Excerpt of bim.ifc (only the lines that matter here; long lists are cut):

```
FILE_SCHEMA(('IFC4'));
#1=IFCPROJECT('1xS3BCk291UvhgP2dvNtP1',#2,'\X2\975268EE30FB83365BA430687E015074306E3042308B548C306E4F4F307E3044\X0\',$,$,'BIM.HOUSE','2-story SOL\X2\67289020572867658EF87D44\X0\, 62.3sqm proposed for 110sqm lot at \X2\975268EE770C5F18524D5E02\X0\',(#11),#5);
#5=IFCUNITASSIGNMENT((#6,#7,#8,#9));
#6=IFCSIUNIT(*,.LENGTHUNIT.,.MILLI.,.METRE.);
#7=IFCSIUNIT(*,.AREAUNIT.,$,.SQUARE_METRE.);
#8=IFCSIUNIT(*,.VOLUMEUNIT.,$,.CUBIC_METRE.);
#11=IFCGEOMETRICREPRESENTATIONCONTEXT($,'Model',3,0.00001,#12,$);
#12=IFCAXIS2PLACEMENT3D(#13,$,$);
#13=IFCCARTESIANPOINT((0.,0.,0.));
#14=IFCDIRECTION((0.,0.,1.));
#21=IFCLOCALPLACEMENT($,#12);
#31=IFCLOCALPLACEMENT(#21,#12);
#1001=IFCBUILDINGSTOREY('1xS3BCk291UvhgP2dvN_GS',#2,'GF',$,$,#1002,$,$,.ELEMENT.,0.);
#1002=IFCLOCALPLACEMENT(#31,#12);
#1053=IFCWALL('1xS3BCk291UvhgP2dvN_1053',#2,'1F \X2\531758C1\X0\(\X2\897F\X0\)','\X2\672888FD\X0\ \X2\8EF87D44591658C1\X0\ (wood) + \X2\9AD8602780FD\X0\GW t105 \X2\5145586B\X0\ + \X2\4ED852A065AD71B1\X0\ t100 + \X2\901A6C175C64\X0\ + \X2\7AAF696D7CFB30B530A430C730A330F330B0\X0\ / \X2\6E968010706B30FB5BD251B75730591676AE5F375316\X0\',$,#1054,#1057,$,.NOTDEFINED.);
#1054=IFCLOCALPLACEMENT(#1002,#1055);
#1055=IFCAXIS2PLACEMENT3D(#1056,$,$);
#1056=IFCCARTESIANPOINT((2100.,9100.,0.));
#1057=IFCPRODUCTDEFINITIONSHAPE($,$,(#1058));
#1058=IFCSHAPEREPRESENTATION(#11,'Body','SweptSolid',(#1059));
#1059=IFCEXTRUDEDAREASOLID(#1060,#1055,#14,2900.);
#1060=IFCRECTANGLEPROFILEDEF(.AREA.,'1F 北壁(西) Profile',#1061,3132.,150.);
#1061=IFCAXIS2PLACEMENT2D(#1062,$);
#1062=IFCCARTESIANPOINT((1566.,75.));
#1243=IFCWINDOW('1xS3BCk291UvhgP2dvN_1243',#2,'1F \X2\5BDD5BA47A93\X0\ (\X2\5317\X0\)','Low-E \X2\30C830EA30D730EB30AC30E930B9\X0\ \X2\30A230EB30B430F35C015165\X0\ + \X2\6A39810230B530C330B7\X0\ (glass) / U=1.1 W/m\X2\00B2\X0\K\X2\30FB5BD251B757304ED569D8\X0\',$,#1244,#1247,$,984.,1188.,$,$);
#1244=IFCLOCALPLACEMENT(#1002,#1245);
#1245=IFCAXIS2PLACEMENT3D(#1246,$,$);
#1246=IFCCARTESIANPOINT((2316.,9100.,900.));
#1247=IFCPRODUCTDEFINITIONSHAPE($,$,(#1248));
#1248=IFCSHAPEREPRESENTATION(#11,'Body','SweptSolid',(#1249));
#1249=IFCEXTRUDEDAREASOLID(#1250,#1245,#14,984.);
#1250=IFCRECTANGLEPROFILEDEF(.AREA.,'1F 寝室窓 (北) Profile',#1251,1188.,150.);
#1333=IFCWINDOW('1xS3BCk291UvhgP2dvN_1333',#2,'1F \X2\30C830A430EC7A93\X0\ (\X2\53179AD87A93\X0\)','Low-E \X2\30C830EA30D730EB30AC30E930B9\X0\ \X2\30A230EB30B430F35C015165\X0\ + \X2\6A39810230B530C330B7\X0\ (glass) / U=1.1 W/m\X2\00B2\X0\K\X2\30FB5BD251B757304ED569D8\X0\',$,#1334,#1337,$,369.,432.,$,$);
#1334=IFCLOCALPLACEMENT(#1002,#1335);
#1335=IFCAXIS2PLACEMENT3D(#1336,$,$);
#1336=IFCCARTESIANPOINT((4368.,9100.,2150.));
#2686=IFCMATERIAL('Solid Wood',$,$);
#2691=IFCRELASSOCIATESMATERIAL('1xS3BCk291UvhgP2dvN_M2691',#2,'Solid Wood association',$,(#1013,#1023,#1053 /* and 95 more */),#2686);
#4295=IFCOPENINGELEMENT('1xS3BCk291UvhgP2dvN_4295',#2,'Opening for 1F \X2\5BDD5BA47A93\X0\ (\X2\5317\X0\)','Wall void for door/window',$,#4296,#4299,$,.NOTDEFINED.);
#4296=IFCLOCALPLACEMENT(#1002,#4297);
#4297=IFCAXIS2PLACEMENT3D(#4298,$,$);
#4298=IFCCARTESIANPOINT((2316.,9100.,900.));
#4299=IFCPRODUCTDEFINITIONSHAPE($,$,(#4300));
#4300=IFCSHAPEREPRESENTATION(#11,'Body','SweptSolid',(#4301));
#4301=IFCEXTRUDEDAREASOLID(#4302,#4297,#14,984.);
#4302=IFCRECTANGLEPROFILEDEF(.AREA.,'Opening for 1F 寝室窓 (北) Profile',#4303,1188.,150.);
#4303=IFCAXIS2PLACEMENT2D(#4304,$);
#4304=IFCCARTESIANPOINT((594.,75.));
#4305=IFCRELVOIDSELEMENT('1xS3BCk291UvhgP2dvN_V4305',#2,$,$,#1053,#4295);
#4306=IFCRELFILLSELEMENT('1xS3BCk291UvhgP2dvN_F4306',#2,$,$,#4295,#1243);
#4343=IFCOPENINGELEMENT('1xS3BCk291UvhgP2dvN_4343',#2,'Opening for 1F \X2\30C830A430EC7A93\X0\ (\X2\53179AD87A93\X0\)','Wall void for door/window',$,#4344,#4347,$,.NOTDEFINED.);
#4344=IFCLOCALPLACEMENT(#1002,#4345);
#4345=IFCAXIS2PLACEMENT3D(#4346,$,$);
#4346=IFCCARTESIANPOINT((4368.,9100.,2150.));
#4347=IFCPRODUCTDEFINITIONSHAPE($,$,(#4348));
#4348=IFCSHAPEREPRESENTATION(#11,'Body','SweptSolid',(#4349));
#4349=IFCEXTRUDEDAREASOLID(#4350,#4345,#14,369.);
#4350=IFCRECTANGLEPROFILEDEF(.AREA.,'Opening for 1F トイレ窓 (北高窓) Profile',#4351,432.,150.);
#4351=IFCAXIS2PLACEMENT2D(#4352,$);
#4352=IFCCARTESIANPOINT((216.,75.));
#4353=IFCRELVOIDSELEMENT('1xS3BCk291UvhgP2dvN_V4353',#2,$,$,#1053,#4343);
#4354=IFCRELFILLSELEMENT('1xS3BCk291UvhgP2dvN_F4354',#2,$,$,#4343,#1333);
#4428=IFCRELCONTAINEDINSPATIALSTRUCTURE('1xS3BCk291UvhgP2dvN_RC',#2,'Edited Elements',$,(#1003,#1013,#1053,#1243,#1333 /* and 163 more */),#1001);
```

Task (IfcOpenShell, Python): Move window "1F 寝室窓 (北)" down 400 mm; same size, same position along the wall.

```python
import numpy as np
import ifcopenshell
import ifcopenshell.api.geometry
import ifcopenshell.util.placement
import ifcopenshell.util.unit

model = ifcopenshell.open("bim.ifc")
unit_scale = ifcopenshell.util.unit.calculate_unit_scale(model)

window = model.by_id(1243)
opening = window.FillsVoids[0].RelatingOpeningElement
dz = -0.4 / unit_scale

shift = np.array([0.0, 0.0, dz])
# The window is not placed relative to its opening, so move both.
for product in (opening, window):
    matrix = ifcopenshell.util.placement.get_local_placement(product.ObjectPlacement)
    matrix[:3, 3] += shift
    ifcopenshell.api.geometry.edit_object_placement(model, product=product, matrix=matrix, is_si=False)

print(f"moved by {dz * unit_scale:+.3f} m")

model.write("bim-out.ifc")
```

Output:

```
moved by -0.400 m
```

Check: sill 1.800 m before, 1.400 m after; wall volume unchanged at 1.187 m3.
